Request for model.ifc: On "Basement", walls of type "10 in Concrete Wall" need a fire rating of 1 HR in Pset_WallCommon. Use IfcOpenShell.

First a look at what the model holds.

```python
import ifcopenshell
import ifcopenshell.util.element

model = ifcopenshell.open("model.ifc")
print(model.schema)
storey = next(s for s in model.by_type("IfcBuildingStorey") if s.Name == "Basement")
walls = [e for e in ifcopenshell.util.element.get_decomposition(storey) if e.is_a("IfcWall")]
seen = {}
for e in walls:
    element_type = ifcopenshell.util.element.get_type(e)
    key = (element_type.Name if element_type != e and element_type else None, ifcopenshell.util.element.get_pset(e, "Pset_WallCommon", "FireRating"))
    seen[key] = seen.get(key, 0) + 1
for (name, value), count in sorted(seen.items(), key=str):
    print(count, "x", name, "|", value)
```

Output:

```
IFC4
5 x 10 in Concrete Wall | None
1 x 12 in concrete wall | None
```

```python
import ifcopenshell
import ifcopenshell.api.pset
import ifcopenshell.util.element

model = ifcopenshell.open("model.ifc")

storey = next(s for s in model.by_type("IfcBuildingStorey") if s.Name == "Basement")
walls = [e for e in ifcopenshell.util.element.get_decomposition(storey) if e.is_a("IfcWall")]

count = 0
for e in walls:
    element_type = ifcopenshell.util.element.get_type(e)
    if element_type in (None, e) or element_type.Name != "10 in Concrete Wall":
        continue
    # add_pset returns the element's existing set when there is one.
    pset = ifcopenshell.api.pset.add_pset(model, product=e, name="Pset_WallCommon")
    ifcopenshell.api.pset.edit_pset(model, pset=pset, properties={"FireRating": "1 HR"})
    count += 1

print(count, "walls updated")

model.write("model_updated.ifc")
```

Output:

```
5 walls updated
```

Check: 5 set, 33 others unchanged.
